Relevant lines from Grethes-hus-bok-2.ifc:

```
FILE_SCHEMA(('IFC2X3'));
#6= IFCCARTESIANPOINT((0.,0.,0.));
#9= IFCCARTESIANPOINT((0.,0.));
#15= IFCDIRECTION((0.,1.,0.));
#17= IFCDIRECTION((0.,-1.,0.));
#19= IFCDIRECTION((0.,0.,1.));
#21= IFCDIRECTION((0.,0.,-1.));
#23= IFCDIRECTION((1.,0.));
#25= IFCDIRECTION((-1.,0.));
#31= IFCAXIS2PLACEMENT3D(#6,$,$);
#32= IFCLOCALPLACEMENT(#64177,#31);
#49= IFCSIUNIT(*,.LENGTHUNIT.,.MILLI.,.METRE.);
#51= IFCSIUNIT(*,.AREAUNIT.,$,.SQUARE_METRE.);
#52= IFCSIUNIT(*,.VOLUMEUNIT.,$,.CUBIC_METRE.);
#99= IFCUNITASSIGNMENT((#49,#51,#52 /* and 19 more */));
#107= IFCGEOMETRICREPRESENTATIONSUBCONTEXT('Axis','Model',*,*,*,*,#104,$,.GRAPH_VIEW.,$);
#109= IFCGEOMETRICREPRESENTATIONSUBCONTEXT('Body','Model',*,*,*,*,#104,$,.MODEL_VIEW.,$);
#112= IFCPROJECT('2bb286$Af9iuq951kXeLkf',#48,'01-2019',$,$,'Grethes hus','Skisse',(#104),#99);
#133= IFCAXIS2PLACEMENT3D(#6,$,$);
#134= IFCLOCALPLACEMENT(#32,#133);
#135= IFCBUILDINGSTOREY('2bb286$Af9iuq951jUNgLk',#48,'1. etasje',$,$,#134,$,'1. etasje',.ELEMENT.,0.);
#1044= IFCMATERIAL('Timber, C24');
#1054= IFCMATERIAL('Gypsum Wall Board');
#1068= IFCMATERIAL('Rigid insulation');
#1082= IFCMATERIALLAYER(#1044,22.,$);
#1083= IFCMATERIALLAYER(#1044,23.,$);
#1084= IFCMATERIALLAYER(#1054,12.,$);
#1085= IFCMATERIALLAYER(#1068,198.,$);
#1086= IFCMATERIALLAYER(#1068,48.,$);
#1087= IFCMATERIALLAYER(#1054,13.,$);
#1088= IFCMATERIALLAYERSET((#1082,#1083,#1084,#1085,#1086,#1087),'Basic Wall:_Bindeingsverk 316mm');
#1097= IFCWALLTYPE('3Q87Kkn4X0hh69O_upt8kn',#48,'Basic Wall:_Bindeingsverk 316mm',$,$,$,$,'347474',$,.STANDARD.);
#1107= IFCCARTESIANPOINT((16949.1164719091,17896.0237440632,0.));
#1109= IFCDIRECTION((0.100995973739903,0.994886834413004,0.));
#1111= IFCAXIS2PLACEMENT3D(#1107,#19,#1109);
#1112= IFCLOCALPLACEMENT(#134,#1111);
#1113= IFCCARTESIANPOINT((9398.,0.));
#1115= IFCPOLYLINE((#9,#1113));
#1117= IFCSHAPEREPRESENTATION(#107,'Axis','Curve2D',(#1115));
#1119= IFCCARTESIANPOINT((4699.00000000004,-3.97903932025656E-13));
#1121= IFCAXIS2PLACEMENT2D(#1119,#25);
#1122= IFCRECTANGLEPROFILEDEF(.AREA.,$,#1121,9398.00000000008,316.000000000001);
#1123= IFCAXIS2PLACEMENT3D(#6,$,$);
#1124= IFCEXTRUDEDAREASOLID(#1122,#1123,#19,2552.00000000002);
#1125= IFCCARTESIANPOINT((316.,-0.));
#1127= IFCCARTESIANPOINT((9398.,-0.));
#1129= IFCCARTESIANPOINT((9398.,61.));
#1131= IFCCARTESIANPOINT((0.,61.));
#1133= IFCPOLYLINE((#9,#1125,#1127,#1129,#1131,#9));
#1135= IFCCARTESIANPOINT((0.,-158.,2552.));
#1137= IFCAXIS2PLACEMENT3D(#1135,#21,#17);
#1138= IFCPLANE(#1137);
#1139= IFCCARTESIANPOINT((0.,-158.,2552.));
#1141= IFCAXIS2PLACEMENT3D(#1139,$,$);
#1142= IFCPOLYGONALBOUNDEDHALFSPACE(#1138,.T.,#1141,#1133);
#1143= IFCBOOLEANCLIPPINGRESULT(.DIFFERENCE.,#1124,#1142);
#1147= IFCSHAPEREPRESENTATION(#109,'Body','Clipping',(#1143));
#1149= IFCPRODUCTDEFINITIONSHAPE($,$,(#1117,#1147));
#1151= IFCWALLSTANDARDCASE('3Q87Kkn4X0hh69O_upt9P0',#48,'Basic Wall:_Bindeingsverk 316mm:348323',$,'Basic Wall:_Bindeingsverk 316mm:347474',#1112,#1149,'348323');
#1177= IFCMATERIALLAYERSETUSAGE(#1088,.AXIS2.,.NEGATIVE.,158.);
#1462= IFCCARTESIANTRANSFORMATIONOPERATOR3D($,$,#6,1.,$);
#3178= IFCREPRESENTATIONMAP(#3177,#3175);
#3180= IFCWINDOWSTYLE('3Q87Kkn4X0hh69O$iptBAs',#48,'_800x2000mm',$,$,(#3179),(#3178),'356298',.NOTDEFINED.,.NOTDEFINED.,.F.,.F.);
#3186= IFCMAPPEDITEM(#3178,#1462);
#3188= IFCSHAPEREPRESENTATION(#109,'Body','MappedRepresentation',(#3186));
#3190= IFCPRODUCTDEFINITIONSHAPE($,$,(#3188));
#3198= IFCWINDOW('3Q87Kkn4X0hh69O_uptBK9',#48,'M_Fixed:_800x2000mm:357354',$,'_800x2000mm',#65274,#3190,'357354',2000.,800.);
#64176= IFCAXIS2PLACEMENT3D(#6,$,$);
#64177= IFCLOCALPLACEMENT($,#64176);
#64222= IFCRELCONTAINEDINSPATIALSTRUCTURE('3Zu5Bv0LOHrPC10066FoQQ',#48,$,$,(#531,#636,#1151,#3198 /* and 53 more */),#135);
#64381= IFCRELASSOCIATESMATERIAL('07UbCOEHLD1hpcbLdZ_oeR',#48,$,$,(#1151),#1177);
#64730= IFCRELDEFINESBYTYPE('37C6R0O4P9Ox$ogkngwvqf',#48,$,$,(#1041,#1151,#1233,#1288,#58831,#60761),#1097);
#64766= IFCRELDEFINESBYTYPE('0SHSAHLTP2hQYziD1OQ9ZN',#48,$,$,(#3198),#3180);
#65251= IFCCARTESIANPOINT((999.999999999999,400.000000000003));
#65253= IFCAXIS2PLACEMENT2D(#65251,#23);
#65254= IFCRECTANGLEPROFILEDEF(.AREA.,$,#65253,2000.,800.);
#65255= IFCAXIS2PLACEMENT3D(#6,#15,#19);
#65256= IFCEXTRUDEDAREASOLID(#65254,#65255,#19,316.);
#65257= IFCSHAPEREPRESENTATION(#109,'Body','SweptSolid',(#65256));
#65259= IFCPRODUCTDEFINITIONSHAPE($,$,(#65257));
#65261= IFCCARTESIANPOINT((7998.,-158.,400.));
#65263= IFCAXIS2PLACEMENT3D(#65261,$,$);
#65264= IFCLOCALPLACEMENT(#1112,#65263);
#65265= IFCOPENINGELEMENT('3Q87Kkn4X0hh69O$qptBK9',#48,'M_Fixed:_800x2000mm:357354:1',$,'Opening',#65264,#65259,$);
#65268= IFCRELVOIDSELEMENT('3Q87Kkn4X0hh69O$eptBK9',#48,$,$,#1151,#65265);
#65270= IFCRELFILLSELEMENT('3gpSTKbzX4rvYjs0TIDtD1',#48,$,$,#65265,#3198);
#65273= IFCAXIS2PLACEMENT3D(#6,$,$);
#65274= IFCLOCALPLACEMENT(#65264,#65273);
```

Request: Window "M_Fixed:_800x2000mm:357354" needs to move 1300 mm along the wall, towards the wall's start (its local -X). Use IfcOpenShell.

```python
import ifcopenshell
import ifcopenshell.api.geometry
import ifcopenshell.util.placement
import ifcopenshell.util.unit

model = ifcopenshell.open("Grethes-hus-bok-2.ifc")
unit_scale = ifcopenshell.util.unit.calculate_unit_scale(model)

window = model.by_guid("3Q87Kkn4X0hh69O_uptBK9")
opening = window.FillsVoids[0].RelatingOpeningElement
wall = opening.VoidsElements[0].RelatingBuildingElement

wall_matrix = ifcopenshell.util.placement.get_local_placement(wall.ObjectPlacement)
shift = wall_matrix[:3, 0] * -1.3 / unit_scale
before = ifcopenshell.util.placement.get_local_placement(window.ObjectPlacement)[:3, 3].copy()

# The window is placed relative to its opening, so it follows when the opening moves.
matrix = ifcopenshell.util.placement.get_local_placement(opening.ObjectPlacement)
matrix[:3, 3] += shift
ifcopenshell.api.geometry.edit_object_placement(
    model, product=opening, matrix=matrix, is_si=False, should_transform_children=True
)

after = ifcopenshell.util.placement.get_local_placement(window.ObjectPlacement)[:3, 3]
print("window moved by", (after - before).round(3) + 0.0)

model.write("Grethes-hus-bok-2_updated.ifc")
```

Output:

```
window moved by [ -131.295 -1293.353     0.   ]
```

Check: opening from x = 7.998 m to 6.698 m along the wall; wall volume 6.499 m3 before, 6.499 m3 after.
